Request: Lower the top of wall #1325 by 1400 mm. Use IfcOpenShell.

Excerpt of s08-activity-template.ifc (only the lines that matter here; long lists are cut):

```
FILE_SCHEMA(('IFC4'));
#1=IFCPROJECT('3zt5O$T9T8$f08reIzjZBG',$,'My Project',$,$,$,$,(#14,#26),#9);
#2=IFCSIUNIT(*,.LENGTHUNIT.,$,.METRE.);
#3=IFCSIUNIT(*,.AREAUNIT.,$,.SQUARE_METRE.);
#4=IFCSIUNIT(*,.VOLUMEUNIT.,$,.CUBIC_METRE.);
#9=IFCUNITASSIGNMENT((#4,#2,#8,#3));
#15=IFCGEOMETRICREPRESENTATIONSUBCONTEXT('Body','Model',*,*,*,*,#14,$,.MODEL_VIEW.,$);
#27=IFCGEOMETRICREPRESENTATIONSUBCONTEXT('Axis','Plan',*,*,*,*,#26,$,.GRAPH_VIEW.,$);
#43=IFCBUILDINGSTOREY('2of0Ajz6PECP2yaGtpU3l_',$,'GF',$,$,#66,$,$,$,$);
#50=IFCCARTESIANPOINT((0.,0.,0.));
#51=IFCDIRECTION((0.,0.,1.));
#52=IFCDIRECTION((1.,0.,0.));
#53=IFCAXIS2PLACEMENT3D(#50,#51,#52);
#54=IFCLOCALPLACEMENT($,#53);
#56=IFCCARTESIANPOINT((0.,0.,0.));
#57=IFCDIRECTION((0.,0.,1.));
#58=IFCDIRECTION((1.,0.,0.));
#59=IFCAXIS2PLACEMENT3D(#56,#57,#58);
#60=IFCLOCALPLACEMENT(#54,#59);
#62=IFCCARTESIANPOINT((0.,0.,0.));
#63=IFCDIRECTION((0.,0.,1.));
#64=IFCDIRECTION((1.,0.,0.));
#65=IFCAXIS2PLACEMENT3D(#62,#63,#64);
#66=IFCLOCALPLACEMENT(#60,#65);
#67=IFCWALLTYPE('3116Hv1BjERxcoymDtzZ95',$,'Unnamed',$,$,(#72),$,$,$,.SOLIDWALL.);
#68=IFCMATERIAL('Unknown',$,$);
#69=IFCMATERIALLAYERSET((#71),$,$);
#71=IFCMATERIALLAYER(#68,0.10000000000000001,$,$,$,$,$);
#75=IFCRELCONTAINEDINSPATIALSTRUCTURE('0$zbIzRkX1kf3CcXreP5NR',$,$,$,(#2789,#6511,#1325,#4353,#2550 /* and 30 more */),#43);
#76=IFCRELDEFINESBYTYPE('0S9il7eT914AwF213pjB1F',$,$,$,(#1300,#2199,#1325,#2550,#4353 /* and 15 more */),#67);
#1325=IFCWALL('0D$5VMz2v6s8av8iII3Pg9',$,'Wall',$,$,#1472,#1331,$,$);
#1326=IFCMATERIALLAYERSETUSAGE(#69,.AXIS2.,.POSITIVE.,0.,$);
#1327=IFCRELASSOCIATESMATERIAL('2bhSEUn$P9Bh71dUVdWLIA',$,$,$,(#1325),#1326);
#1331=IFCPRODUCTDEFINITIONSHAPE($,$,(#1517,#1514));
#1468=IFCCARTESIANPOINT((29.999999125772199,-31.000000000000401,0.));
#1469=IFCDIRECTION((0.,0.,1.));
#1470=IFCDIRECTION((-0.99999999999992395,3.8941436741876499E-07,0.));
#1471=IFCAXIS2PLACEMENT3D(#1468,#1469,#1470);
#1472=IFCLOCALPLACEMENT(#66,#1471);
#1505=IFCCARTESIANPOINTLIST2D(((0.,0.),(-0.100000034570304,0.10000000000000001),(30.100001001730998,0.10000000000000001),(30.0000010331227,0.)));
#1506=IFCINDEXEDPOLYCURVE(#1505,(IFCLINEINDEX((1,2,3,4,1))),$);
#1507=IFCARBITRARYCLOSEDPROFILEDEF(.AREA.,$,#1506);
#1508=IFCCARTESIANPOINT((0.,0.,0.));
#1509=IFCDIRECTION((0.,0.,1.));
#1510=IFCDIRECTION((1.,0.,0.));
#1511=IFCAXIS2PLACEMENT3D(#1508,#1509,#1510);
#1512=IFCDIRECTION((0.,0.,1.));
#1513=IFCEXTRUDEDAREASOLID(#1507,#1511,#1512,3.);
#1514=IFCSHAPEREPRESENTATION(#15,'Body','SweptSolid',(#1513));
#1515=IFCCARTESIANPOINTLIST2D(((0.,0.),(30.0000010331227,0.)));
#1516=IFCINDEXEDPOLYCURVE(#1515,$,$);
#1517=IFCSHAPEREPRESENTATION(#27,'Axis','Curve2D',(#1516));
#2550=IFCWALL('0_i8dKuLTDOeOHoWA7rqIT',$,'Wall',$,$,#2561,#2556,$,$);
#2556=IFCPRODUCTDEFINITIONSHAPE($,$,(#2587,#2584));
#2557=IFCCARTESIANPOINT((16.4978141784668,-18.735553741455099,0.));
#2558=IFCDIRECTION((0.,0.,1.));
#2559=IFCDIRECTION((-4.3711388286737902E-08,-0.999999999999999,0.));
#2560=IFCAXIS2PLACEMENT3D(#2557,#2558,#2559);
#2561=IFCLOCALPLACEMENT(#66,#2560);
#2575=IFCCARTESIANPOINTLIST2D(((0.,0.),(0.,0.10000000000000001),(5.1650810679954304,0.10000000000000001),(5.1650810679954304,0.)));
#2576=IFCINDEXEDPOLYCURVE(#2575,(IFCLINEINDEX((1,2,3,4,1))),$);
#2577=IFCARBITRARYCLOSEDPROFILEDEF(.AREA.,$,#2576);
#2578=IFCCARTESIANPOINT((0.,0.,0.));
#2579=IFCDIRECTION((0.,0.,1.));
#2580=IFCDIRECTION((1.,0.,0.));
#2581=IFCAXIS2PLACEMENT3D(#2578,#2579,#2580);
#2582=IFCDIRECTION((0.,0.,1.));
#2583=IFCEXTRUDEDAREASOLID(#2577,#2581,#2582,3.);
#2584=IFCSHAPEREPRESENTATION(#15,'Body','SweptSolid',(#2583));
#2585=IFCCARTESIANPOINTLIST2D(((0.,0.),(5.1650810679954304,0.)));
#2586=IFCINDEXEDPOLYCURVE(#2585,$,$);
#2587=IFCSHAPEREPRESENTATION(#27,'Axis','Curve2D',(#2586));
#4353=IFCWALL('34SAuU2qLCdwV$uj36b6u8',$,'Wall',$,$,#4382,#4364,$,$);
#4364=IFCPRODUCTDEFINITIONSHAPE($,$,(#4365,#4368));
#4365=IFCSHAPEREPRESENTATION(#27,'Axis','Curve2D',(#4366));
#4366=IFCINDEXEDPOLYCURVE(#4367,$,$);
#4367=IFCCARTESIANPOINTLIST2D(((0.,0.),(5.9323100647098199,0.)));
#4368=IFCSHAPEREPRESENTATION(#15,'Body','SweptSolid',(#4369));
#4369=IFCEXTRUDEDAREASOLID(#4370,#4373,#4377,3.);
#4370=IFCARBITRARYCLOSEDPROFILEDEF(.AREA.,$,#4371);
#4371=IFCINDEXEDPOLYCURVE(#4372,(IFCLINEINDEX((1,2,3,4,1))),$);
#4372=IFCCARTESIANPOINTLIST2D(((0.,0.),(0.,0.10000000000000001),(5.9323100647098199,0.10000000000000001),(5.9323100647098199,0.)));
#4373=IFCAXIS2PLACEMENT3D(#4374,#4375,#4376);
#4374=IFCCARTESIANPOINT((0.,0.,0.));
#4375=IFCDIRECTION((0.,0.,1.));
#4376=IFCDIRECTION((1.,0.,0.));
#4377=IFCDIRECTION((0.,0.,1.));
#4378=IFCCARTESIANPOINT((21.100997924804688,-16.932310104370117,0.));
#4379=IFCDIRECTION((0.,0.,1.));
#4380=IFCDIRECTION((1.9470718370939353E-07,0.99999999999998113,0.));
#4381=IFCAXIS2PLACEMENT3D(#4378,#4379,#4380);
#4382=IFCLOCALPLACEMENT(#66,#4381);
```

```python
import ifcopenshell
import ifcopenshell.geom
import ifcopenshell.util.representation
import ifcopenshell.util.shape

model = ifcopenshell.open("s08-activity-template.ifc")
settings = ifcopenshell.geom.settings()


def volume(element):
    """Net volume in cubic metres, openings subtracted."""
    shape = ifcopenshell.geom.create_shape(settings, element)
    return ifcopenshell.util.shape.get_volume(shape.geometry)


wall = model.by_id(1325)
before = volume(wall)

body = ifcopenshell.util.representation.get_representation(wall, "Model", "Body")
solid = body.Items[0]
old_height = solid.Depth
solid.Depth -= 1.4
after = volume(wall)

print(f"height {old_height:g} -> {solid.Depth:g}, volume {before:.3f} -> {after:.3f} m3")

model.write("s08-activity-template-out.ifc")
```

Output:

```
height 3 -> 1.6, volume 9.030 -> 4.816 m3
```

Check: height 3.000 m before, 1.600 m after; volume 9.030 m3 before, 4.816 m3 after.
